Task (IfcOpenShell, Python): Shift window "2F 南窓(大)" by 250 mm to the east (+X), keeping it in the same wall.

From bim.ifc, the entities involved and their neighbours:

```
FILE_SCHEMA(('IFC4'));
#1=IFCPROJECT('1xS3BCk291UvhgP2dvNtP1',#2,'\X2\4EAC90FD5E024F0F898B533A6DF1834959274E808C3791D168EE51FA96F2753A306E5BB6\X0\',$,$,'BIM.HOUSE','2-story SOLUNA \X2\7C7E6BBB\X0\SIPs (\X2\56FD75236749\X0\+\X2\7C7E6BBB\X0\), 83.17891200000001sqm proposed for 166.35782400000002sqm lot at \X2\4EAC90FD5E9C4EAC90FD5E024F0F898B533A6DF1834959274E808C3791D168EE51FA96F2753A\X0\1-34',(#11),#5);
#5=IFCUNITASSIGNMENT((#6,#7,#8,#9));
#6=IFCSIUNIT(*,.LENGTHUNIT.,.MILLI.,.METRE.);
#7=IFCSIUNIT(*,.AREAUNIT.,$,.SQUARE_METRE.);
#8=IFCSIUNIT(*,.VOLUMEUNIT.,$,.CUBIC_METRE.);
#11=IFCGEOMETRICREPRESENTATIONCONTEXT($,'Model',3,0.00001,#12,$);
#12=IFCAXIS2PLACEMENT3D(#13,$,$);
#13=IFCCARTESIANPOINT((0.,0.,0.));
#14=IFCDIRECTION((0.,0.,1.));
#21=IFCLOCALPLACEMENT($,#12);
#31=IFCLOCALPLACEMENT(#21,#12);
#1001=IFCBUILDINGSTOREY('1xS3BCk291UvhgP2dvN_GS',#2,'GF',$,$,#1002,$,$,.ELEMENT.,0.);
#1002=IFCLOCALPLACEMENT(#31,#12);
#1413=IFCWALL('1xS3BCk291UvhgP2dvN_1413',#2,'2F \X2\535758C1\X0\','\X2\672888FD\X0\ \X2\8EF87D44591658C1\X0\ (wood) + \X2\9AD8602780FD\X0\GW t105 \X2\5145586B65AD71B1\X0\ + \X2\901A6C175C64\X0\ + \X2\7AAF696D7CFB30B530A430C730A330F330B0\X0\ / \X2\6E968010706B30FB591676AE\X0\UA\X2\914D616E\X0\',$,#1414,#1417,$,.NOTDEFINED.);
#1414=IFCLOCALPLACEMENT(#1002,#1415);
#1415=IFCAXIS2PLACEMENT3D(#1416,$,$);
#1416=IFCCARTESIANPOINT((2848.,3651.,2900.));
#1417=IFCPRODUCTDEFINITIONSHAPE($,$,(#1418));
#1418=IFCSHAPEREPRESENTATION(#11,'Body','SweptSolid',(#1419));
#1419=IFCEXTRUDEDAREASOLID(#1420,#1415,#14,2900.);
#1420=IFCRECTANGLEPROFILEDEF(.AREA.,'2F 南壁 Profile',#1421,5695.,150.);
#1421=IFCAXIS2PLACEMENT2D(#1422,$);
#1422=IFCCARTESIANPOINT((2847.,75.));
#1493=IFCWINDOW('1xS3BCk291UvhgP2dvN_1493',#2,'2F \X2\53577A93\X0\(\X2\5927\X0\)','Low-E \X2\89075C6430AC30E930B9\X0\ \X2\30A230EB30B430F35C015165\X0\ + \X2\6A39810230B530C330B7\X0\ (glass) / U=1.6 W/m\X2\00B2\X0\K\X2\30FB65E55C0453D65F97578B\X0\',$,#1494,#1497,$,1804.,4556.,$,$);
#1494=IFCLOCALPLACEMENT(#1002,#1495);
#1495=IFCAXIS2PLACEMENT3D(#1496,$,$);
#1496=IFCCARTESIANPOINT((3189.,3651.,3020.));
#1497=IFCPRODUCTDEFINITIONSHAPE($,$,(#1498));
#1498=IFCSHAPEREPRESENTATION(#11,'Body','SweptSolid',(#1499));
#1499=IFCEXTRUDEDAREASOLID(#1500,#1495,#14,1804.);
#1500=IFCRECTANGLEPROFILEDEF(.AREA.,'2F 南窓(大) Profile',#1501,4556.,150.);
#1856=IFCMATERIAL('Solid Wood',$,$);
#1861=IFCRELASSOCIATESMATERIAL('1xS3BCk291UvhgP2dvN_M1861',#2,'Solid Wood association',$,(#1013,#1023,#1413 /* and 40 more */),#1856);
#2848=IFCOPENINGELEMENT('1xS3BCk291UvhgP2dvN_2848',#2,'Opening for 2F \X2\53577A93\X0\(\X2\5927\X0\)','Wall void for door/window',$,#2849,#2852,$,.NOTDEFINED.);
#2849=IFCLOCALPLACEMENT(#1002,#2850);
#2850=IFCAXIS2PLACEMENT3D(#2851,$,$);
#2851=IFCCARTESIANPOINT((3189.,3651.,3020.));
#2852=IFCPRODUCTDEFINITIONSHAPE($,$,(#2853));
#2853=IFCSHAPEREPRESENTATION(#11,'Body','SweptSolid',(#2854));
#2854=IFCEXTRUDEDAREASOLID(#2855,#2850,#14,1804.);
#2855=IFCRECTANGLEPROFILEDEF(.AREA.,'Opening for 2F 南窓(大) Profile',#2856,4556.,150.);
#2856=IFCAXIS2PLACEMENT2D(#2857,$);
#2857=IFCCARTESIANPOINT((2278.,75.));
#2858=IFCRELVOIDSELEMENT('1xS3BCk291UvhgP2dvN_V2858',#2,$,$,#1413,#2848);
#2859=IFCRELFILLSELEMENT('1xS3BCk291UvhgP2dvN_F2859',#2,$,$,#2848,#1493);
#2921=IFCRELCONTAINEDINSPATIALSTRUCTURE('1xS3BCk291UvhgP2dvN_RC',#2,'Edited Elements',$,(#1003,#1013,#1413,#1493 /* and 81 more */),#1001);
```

```python
import ifcopenshell
import ifcopenshell.api.geometry
import ifcopenshell.util.placement
import ifcopenshell.util.unit

model = ifcopenshell.open("bim.ifc")
unit_scale = ifcopenshell.util.unit.calculate_unit_scale(model)

window = model.by_guid("1xS3BCk291UvhgP2dvN_1493")
opening = window.FillsVoids[0].RelatingOpeningElement
wall = opening.VoidsElements[0].RelatingBuildingElement

wall_matrix = ifcopenshell.util.placement.get_local_placement(wall.ObjectPlacement)
shift = wall_matrix[:3, 0] * 0.25 / unit_scale
before = ifcopenshell.util.placement.get_local_placement(window.ObjectPlacement)[:3, 3].copy()

# The window is not placed relative to its opening, so move both.
for product in (opening, window):
    matrix = ifcopenshell.util.placement.get_local_placement(product.ObjectPlacement)
    matrix[:3, 3] += shift
    ifcopenshell.api.geometry.edit_object_placement(model, product=product, matrix=matrix, is_si=False)

after = ifcopenshell.util.placement.get_local_placement(window.ObjectPlacement)[:3, 3]
print("window moved by", (after - before).round(3) + 0.0)

model.write("bim_rev.ifc")
```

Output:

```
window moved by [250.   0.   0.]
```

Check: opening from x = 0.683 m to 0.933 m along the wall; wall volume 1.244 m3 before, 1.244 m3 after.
